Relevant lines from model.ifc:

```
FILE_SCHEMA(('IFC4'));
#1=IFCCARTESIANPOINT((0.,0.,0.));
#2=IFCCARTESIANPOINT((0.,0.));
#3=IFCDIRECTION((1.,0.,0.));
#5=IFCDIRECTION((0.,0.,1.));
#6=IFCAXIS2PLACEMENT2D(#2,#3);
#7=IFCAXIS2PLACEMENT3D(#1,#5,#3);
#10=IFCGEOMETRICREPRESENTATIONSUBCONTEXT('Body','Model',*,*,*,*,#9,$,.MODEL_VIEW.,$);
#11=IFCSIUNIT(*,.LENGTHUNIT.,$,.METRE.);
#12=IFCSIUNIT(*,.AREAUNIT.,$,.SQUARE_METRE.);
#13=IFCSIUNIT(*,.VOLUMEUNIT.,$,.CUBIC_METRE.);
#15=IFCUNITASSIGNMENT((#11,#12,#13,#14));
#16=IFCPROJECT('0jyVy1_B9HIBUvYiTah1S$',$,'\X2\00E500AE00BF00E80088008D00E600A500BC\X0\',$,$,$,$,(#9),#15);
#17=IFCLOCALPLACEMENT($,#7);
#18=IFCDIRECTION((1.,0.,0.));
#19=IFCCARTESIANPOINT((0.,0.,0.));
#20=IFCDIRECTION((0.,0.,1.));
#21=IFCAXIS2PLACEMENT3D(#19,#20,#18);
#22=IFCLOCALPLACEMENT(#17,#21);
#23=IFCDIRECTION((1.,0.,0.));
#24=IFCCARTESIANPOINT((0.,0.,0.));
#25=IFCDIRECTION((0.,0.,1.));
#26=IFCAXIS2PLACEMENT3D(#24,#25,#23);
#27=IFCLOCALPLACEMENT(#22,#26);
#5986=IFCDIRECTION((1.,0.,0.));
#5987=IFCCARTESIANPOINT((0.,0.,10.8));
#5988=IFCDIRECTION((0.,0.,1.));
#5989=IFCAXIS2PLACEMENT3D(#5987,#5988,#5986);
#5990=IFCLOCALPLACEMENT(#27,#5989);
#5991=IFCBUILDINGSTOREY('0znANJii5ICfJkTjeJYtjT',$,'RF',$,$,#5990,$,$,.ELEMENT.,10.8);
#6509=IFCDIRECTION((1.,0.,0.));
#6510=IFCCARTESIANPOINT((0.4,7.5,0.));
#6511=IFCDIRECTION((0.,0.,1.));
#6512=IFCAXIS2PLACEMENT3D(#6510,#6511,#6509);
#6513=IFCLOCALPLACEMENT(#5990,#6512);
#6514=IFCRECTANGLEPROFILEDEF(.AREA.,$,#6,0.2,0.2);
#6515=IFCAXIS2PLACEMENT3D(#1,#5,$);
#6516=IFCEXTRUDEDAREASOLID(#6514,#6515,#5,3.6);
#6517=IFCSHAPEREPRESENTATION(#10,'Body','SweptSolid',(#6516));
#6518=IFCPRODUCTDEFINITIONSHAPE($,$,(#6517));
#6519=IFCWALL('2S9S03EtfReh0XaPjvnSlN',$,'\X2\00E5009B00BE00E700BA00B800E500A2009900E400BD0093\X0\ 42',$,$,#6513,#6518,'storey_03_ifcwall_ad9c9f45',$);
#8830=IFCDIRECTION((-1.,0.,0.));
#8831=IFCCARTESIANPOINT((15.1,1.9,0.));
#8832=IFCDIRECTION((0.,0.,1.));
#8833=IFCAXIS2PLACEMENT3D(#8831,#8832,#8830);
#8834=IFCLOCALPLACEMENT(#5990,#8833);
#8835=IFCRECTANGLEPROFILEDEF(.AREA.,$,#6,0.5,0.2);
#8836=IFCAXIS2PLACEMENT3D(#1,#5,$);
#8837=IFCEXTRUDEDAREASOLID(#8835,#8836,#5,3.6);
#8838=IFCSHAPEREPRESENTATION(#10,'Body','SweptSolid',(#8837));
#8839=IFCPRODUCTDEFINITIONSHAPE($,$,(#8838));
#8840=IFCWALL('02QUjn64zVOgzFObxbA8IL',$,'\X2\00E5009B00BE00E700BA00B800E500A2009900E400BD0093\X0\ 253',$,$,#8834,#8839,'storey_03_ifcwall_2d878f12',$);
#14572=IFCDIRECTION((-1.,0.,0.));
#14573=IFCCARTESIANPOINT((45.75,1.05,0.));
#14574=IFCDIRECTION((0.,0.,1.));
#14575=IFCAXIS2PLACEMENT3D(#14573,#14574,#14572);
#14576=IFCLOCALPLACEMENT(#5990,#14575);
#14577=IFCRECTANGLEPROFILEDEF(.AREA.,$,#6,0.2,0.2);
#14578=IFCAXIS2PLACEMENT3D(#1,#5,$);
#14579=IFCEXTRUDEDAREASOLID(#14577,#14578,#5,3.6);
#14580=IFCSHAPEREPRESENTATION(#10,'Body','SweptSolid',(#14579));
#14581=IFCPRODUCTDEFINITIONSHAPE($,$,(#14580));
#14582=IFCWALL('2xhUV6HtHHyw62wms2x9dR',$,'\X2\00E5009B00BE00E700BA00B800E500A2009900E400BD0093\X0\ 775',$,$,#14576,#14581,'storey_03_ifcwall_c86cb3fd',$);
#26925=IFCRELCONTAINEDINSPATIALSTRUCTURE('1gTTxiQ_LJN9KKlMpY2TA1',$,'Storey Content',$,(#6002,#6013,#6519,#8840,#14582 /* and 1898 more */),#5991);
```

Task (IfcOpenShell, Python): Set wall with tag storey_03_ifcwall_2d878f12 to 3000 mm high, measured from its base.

```python
import ifcopenshell
import ifcopenshell.geom
import ifcopenshell.util.representation
import ifcopenshell.util.shape

model = ifcopenshell.open("model.ifc")
settings = ifcopenshell.geom.settings()


def volume(element):
    """Net volume in cubic metres, openings subtracted."""
    shape = ifcopenshell.geom.create_shape(settings, element)
    return ifcopenshell.util.shape.get_volume(shape.geometry)


wall = model.by_guid("02QUjn64zVOgzFObxbA8IL")
before = volume(wall)

body = ifcopenshell.util.representation.get_representation(wall, "Model", "Body")
solid = body.Items[0]
old_height = solid.Depth
solid.Depth = 3.0
after = volume(wall)

print(f"height {old_height:g} -> {solid.Depth:g}, volume {before:.3f} -> {after:.3f} m3")

model.write("model_v2.ifc")
```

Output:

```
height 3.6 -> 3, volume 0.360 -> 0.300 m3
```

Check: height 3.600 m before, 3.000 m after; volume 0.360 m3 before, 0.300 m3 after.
